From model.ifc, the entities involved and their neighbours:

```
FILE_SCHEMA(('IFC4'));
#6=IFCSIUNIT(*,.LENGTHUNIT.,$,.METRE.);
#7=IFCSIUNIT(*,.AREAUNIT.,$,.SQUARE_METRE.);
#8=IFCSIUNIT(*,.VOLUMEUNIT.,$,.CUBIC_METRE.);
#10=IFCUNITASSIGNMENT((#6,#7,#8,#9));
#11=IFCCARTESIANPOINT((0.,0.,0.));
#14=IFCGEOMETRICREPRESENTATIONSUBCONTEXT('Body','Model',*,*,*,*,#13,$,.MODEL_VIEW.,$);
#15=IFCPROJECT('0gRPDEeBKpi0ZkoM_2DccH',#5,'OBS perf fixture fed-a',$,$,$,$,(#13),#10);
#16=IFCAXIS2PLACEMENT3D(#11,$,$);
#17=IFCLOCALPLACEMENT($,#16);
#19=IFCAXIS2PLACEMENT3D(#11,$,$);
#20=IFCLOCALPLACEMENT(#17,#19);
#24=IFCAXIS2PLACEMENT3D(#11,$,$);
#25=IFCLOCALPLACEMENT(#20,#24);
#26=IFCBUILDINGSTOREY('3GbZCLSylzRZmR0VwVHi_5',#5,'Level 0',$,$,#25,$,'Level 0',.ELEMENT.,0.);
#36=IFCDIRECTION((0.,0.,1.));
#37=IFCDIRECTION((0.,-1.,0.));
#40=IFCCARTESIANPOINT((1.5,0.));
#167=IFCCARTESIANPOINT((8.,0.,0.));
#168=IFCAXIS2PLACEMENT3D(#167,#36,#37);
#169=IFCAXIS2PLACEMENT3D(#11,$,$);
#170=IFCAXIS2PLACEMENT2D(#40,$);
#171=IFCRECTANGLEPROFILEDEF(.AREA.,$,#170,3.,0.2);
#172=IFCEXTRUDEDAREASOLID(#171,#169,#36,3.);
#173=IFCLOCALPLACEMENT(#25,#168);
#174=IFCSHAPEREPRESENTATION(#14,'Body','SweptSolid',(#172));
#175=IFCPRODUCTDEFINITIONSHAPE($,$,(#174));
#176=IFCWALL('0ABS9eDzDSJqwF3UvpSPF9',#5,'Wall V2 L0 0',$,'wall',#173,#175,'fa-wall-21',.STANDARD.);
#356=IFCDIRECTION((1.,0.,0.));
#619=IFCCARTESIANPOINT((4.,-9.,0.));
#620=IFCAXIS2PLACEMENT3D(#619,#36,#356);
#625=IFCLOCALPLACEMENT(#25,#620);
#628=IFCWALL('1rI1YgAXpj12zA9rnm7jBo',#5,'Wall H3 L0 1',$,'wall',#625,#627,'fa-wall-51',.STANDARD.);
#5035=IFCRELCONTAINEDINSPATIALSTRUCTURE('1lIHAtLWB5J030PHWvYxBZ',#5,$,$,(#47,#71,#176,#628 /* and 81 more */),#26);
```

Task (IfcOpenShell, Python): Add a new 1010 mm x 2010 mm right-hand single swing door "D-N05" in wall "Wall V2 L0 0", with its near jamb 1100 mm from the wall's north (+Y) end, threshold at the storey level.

```python
import numpy as np
import ifcopenshell
import ifcopenshell.api.feature
import ifcopenshell.api.geometry
import ifcopenshell.api.root
import ifcopenshell.api.spatial
import ifcopenshell.geom
import ifcopenshell.util.element
import ifcopenshell.util.placement
import ifcopenshell.util.representation
import ifcopenshell.util.shape
import ifcopenshell.util.unit

model = ifcopenshell.open("model.ifc")
unit_scale = ifcopenshell.util.unit.calculate_unit_scale(model)
settings = ifcopenshell.geom.settings()


def volume(element):
    """Net volume in cubic metres, openings subtracted."""
    shape = ifcopenshell.geom.create_shape(settings, element)
    return ifcopenshell.util.shape.get_volume(shape.geometry)


wall = model.by_id(176)
storey = ifcopenshell.util.element.get_container(wall, ifc_class="IfcBuildingStorey")
context = ifcopenshell.util.representation.get_context(model, "Model", "Body", "MODEL_VIEW")
before = volume(wall)

width, height, from_end, sill = 1.01, 2.01, 1.1, 0.0  # metres

# The wall runs along its own X axis, and the end named is its -X end.
wall_shape = ifcopenshell.geom.create_shape(settings, wall)
x, y, z = ifcopenshell.util.shape.get_vertices(wall_shape.geometry).T
start = x.min() + from_end
face, thickness = float(y.min()), float(y.max() - y.min())
wall_matrix = ifcopenshell.util.placement.get_local_placement(wall.ObjectPlacement)
level = ifcopenshell.util.placement.get_local_placement(storey.ObjectPlacement)[2, 3]


def in_wall(x, y):
    """Placement at x, y metres in the wall's axes, at sill height."""
    matrix = wall_matrix.copy()
    matrix[:, 3] = wall_matrix @ np.array([x / unit_scale, y / unit_scale, 0.0, 1.0])
    matrix[2, 3] = level + sill / unit_scale
    return matrix


# Opening: a box that overshoots both wall faces by 50 mm.
opening = ifcopenshell.api.root.create_entity(model, ifc_class="IfcOpeningElement", predefined_type="OPENING")
box = ifcopenshell.api.geometry.add_wall_representation(
    model, context=context, length=width, height=height, thickness=thickness + 0.1
)
ifcopenshell.api.geometry.assign_representation(model, product=opening, representation=box)
ifcopenshell.api.geometry.edit_object_placement(model, product=opening, matrix=in_wall(start, face - 0.05), is_si=False)
ifcopenshell.api.feature.add_feature(model, feature=opening, element=wall)

door = ifcopenshell.api.root.create_entity(model, ifc_class="IfcDoor", name="D-N05", predefined_type="DOOR")
door.OverallWidth, door.OverallHeight = width / unit_scale, height / unit_scale
door.OperationType = "SINGLE_SWING_RIGHT"
body = ifcopenshell.api.geometry.add_door_representation(
    model,
    context=context,
    overall_width=door.OverallWidth,
    overall_height=door.OverallHeight,
    operation_type="SINGLE_SWING_RIGHT",
    lining_properties={"LiningDepth": thickness / unit_scale, "ThresholdDepth": thickness / unit_scale},
)
ifcopenshell.api.geometry.assign_representation(model, product=door, representation=body)
ifcopenshell.api.spatial.assign_container(model, products=[door], relating_structure=storey)
ifcopenshell.api.feature.add_filling(model, opening=opening, element=door)

# The lining spans the wall, so the door starts at the wall face.
ifcopenshell.api.geometry.edit_object_placement(model, product=door, matrix=in_wall(start, face), is_si=False)

after = volume(wall)

print(f"wall volume {before:.3f} -> {after:.3f} m3")

model.write("model_v2.ifc")
```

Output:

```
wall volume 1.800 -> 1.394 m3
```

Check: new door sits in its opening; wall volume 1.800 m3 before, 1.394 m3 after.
